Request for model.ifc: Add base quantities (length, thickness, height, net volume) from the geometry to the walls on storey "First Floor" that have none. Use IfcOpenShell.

First a look at what the model holds.

```python
import ifcopenshell
import ifcopenshell.util.element
import ifcopenshell.util.unit

model = ifcopenshell.open("model.ifc")
print(model.schema)
for unit_type in ("LENGTHUNIT", "AREAUNIT", "VOLUMEUNIT"):
    print(unit_type, ifcopenshell.util.unit.calculate_unit_scale(model, unit_type))
storey = next(s for s in model.by_type("IfcBuildingStorey") if s.Name == "First Floor")
walls = [e for e in ifcopenshell.util.element.get_decomposition(storey) if e.is_a("IfcWall")]
for e in sorted(walls, key=lambda e: e.id()):
    print(e.id(), e.is_a(), e.Name, list(ifcopenshell.util.element.get_psets(e, qtos_only=True)), sep=" | ")
```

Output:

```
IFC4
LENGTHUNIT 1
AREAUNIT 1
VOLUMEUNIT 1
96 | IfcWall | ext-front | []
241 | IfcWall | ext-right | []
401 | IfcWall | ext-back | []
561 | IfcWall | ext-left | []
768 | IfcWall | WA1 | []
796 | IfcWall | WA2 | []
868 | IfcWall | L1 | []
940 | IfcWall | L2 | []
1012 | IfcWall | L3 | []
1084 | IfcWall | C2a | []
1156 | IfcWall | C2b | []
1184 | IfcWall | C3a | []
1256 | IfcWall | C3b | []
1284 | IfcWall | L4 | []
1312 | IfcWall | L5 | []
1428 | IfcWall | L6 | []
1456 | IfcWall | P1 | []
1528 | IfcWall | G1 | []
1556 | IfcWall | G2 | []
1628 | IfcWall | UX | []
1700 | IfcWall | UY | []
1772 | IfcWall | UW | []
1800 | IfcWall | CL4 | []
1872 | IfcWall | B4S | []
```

```python
import ifcopenshell
import ifcopenshell.api.pset
import ifcopenshell.geom
import ifcopenshell.util.element
import ifcopenshell.util.shape
import ifcopenshell.util.unit

model = ifcopenshell.open("model.ifc")
unit_scale = ifcopenshell.util.unit.calculate_unit_scale(model)
volume_scale = ifcopenshell.util.unit.calculate_unit_scale(model, "VOLUMEUNIT")
settings = ifcopenshell.geom.settings()

storey = next(s for s in model.by_type("IfcBuildingStorey") if s.Name == "First Floor")
walls = [e for e in ifcopenshell.util.element.get_decomposition(storey) if e.is_a("IfcWall")]

for e in sorted(walls, key=lambda e: e.id()):
    if ifcopenshell.util.element.get_psets(e, qtos_only=True, should_inherit=False):
        continue
    # Geometry comes back in metres, in the element's own axes.
    shape = ifcopenshell.geom.create_shape(settings, e)
    values = {
        "Length": ifcopenshell.util.shape.get_x(shape.geometry) / unit_scale,
        "Width": ifcopenshell.util.shape.get_y(shape.geometry) / unit_scale,
        "Height": ifcopenshell.util.shape.get_z(shape.geometry) / unit_scale,
        "NetVolume": ifcopenshell.util.shape.get_volume(shape.geometry) / volume_scale,
    }
    qto = ifcopenshell.api.pset.add_qto(model, product=e, name="Qto_WallBaseQuantities")
    ifcopenshell.api.pset.edit_qto(model, qto=qto, properties=values)
    print(e.id(), {k: round(v, 3) for k, v in values.items()})

model.write("model-out.ifc")
```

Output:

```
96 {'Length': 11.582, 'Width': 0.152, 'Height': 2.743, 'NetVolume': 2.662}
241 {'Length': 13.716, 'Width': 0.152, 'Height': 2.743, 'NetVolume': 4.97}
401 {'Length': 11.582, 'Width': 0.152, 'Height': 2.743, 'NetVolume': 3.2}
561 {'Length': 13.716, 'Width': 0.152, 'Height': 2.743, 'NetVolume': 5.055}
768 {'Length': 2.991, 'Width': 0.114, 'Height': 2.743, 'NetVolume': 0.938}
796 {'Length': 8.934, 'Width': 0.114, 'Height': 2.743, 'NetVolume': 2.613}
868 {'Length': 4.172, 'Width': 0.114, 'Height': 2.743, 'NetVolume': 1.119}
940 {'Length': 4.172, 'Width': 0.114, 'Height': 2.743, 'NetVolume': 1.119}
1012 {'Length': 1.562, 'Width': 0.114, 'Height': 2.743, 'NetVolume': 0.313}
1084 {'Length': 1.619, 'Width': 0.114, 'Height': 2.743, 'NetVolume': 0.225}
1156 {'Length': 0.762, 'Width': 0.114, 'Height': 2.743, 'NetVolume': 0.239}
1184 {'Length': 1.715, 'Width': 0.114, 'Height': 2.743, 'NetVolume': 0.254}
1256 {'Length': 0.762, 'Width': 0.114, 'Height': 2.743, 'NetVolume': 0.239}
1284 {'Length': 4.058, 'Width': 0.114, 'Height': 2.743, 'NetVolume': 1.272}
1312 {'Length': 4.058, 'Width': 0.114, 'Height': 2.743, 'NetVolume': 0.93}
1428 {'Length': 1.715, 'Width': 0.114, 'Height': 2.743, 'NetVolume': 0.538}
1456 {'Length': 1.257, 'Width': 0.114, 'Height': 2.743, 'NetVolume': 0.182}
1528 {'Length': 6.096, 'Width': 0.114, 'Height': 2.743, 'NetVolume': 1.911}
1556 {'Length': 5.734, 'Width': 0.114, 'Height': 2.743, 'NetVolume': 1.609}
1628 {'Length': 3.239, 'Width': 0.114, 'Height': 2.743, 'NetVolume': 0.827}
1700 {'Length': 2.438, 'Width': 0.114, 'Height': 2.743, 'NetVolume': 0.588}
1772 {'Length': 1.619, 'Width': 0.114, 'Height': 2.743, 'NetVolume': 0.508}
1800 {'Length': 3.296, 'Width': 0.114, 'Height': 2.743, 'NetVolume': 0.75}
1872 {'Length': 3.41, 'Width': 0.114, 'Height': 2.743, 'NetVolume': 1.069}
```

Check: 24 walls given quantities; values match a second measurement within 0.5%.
